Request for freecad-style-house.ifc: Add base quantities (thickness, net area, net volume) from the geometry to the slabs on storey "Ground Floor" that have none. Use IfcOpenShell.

First a look at what the model holds.

```python
import ifcopenshell
import ifcopenshell.util.element
import ifcopenshell.util.unit

model = ifcopenshell.open("freecad-style-house.ifc")
print(model.schema)
for unit_type in ("LENGTHUNIT", "AREAUNIT", "VOLUMEUNIT"):
    print(unit_type, ifcopenshell.util.unit.calculate_unit_scale(model, unit_type))
storey = next(s for s in model.by_type("IfcBuildingStorey") if s.Name == "Ground Floor")
slabs = [e for e in ifcopenshell.util.element.get_decomposition(storey) if e.is_a("IfcSlab")]
for e in sorted(slabs, key=lambda e: e.id()):
    print(e.id(), e.is_a(), e.Name, list(ifcopenshell.util.element.get_psets(e, qtos_only=True)), sep=" | ")
```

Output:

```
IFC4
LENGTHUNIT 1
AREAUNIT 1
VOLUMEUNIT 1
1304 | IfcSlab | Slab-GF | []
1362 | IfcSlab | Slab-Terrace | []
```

```python
import ifcopenshell
import ifcopenshell.api.pset
import ifcopenshell.geom
import ifcopenshell.util.element
import ifcopenshell.util.shape
import ifcopenshell.util.unit

model = ifcopenshell.open("freecad-style-house.ifc")
unit_scale = ifcopenshell.util.unit.calculate_unit_scale(model)
area_scale = ifcopenshell.util.unit.calculate_unit_scale(model, "AREAUNIT")
volume_scale = ifcopenshell.util.unit.calculate_unit_scale(model, "VOLUMEUNIT")
settings = ifcopenshell.geom.settings()

storey = next(s for s in model.by_type("IfcBuildingStorey") if s.Name == "Ground Floor")
slabs = [e for e in ifcopenshell.util.element.get_decomposition(storey) if e.is_a("IfcSlab")]

for e in sorted(slabs, key=lambda e: e.id()):
    if ifcopenshell.util.element.get_psets(e, qtos_only=True, should_inherit=False):
        continue
    # Geometry comes back in metres, in the element's own axes.
    shape = ifcopenshell.geom.create_shape(settings, e)
    values = {
        "Width": ifcopenshell.util.shape.get_z(shape.geometry) / unit_scale,
        "NetArea": ifcopenshell.util.shape.get_footprint_area(shape.geometry) / area_scale,
        "NetVolume": ifcopenshell.util.shape.get_volume(shape.geometry) / volume_scale,
    }
    qto = ifcopenshell.api.pset.add_qto(model, product=e, name="Qto_SlabBaseQuantities")
    ifcopenshell.api.pset.edit_qto(model, qto=qto, properties=values)
    print(e.id(), {k: round(v, 3) for k, v in values.items()})

model.write("freecad-style-house_updated.ifc")
```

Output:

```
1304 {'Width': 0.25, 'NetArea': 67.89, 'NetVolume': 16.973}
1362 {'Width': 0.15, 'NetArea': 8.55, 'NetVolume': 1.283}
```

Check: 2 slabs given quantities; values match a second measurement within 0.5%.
